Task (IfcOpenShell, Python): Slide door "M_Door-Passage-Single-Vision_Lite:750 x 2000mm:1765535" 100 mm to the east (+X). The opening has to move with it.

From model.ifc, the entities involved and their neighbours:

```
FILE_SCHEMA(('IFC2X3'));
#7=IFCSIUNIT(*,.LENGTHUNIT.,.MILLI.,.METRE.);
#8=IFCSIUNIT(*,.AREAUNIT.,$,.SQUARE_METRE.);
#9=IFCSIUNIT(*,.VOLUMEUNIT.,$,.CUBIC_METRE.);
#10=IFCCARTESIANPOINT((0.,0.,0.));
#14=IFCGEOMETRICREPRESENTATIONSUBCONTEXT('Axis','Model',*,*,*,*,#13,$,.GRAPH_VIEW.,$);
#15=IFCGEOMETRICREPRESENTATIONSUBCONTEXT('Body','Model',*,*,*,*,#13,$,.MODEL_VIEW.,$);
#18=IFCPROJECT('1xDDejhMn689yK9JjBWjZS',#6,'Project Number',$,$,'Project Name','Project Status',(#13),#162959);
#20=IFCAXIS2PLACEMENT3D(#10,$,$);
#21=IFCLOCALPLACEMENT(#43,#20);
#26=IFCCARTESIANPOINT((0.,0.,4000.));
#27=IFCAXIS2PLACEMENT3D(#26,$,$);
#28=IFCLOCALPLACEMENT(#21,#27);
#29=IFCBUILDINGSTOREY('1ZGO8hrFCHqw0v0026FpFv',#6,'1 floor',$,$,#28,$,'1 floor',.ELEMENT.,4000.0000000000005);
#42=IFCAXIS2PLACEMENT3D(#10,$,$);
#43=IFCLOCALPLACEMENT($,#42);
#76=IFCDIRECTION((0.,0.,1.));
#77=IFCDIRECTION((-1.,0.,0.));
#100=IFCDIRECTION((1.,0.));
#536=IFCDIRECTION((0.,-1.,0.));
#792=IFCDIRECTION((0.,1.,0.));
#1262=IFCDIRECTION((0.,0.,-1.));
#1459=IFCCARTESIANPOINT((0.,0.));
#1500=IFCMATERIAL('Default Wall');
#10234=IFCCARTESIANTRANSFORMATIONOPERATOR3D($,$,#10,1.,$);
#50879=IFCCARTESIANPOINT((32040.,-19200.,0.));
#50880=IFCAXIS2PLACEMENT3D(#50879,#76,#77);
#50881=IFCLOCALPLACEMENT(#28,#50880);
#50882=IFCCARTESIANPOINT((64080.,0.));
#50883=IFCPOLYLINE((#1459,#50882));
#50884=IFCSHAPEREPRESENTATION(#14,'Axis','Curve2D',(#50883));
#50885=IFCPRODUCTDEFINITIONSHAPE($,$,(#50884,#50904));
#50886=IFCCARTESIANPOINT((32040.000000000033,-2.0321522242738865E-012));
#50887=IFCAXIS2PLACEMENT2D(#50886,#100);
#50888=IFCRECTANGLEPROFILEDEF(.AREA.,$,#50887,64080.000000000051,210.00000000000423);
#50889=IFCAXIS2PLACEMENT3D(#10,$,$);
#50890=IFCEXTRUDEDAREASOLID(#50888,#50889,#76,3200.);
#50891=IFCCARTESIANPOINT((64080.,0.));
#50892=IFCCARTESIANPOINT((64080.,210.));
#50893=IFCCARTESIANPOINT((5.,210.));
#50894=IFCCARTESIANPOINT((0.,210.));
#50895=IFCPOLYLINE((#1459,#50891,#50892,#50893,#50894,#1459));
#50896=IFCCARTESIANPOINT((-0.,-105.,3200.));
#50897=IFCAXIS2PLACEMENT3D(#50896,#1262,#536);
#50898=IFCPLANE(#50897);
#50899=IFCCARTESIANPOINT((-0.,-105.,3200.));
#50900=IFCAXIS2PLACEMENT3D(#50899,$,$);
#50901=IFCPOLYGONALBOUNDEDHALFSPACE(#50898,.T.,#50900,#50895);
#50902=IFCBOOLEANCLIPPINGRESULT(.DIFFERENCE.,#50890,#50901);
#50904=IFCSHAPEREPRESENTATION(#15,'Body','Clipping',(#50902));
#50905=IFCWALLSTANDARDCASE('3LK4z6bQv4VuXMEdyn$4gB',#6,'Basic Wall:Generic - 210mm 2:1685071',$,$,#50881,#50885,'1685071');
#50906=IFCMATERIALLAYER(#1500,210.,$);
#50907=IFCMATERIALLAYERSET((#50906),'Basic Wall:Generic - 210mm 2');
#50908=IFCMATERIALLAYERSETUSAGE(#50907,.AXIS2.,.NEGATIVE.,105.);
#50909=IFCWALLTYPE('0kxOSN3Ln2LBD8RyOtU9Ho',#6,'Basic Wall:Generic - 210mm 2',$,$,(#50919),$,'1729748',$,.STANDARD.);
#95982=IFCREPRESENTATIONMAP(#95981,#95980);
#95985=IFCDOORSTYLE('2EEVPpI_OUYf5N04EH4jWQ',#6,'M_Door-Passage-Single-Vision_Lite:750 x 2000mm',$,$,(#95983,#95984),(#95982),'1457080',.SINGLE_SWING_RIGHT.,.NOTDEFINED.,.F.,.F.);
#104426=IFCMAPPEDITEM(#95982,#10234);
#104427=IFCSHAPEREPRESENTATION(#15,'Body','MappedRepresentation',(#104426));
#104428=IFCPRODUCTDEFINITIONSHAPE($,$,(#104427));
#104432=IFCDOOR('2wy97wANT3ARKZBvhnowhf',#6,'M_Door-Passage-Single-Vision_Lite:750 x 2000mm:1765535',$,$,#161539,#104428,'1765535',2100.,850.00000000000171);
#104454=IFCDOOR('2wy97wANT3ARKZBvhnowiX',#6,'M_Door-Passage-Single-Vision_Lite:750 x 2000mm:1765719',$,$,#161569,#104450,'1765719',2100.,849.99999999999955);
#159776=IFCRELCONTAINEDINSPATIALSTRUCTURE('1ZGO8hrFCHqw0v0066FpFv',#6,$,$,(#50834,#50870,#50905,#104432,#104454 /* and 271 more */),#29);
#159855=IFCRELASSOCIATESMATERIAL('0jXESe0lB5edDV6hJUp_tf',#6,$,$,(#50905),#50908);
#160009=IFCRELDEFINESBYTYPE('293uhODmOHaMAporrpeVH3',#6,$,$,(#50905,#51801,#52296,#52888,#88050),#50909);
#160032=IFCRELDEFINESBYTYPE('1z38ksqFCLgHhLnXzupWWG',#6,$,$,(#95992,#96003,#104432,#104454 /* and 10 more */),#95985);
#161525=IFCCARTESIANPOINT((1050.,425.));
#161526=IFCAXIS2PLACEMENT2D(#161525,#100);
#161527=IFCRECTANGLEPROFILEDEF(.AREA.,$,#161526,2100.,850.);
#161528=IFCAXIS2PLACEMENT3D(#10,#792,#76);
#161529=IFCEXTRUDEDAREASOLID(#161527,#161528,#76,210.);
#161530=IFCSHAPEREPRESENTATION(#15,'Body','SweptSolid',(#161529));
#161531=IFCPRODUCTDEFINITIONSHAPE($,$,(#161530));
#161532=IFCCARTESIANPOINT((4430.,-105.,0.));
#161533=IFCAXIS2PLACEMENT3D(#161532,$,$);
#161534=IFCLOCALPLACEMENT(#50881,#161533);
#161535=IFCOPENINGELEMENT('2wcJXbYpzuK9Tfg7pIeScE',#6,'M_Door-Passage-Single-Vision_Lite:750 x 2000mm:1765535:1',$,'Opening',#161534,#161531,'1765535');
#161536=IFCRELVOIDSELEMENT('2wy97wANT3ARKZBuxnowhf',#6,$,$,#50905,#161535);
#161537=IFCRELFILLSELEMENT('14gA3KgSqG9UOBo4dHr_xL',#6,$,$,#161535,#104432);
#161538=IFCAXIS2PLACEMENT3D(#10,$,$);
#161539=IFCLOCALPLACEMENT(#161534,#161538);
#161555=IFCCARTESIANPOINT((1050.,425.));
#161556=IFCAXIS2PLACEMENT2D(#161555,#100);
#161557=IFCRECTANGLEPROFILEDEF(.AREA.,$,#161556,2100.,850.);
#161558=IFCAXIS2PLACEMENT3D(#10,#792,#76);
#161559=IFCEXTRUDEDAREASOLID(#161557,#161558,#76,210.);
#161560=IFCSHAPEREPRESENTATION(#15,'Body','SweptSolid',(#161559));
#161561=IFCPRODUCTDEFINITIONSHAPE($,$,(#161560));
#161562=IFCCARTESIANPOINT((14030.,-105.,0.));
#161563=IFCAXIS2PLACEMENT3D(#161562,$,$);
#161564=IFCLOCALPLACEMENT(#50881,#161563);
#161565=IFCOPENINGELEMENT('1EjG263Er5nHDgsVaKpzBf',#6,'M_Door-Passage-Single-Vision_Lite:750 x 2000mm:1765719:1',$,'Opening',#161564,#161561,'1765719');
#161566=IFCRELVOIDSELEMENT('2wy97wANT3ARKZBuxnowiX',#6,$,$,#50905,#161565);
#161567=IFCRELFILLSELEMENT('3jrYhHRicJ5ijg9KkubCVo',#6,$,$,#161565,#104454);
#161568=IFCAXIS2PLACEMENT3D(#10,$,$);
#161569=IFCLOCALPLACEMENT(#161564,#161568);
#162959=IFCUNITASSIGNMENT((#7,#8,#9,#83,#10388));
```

```python
import ifcopenshell
import ifcopenshell.api.geometry
import ifcopenshell.util.placement

model = ifcopenshell.open("model.ifc")

door = model.by_guid("2wy97wANT3ARKZBvhnowhf")
opening = door.FillsVoids[0].RelatingOpeningElement
wall = opening.VoidsElements[0].RelatingBuildingElement

wall_matrix = ifcopenshell.util.placement.get_local_placement(wall.ObjectPlacement)
shift = wall_matrix[:3, 0] * -100.0
before = ifcopenshell.util.placement.get_local_placement(door.ObjectPlacement)[:3, 3].copy()

# The door is placed relative to its opening, so it follows when the opening moves.
matrix = ifcopenshell.util.placement.get_local_placement(opening.ObjectPlacement)
matrix[:3, 3] += shift
ifcopenshell.api.geometry.edit_object_placement(
    model, product=opening, matrix=matrix, is_si=False, should_transform_children=True
)

after = ifcopenshell.util.placement.get_local_placement(door.ObjectPlacement)[:3, 3]
print("door moved by", (after - before).round(3) + 0.0)

model.write("model_rev.ifc")
```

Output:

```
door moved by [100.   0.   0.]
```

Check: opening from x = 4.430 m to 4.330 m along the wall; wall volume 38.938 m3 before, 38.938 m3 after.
